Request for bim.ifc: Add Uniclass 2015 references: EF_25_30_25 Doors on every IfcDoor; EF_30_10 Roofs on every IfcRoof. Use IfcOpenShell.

First a look at what the model holds.

```python
import ifcopenshell

model = ifcopenshell.open("bim.ifc")
print(model.schema)
print("classifications:", [c.Name for c in model.by_type("IfcClassification")])
for ifc_class in ("IfcDoor", "IfcRoof", "IfcStair", "IfcWall", "IfcWindow"):
    print(ifc_class, len(model.by_type(ifc_class)))
```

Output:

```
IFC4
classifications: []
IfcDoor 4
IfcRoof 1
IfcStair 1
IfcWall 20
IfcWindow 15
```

```python
import ifcopenshell
import ifcopenshell.api.classification

model = ifcopenshell.open("bim.ifc")

system = ifcopenshell.api.classification.add_classification(model, classification="Uniclass 2015")

codes = {
    "IfcDoor": ("EF_25_30_25", "Doors"),
    "IfcRoof": ("EF_30_10", "Roofs"),
}
for ifc_class, (code, name) in codes.items():
    products = model.by_type(ifc_class)
    ifcopenshell.api.classification.add_reference(
        model, products=products, classification=system, identification=code, name=name
    )
    print(code, len(products))

model.write("bim_rev.ifc")
```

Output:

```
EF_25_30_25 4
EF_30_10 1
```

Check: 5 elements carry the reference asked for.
